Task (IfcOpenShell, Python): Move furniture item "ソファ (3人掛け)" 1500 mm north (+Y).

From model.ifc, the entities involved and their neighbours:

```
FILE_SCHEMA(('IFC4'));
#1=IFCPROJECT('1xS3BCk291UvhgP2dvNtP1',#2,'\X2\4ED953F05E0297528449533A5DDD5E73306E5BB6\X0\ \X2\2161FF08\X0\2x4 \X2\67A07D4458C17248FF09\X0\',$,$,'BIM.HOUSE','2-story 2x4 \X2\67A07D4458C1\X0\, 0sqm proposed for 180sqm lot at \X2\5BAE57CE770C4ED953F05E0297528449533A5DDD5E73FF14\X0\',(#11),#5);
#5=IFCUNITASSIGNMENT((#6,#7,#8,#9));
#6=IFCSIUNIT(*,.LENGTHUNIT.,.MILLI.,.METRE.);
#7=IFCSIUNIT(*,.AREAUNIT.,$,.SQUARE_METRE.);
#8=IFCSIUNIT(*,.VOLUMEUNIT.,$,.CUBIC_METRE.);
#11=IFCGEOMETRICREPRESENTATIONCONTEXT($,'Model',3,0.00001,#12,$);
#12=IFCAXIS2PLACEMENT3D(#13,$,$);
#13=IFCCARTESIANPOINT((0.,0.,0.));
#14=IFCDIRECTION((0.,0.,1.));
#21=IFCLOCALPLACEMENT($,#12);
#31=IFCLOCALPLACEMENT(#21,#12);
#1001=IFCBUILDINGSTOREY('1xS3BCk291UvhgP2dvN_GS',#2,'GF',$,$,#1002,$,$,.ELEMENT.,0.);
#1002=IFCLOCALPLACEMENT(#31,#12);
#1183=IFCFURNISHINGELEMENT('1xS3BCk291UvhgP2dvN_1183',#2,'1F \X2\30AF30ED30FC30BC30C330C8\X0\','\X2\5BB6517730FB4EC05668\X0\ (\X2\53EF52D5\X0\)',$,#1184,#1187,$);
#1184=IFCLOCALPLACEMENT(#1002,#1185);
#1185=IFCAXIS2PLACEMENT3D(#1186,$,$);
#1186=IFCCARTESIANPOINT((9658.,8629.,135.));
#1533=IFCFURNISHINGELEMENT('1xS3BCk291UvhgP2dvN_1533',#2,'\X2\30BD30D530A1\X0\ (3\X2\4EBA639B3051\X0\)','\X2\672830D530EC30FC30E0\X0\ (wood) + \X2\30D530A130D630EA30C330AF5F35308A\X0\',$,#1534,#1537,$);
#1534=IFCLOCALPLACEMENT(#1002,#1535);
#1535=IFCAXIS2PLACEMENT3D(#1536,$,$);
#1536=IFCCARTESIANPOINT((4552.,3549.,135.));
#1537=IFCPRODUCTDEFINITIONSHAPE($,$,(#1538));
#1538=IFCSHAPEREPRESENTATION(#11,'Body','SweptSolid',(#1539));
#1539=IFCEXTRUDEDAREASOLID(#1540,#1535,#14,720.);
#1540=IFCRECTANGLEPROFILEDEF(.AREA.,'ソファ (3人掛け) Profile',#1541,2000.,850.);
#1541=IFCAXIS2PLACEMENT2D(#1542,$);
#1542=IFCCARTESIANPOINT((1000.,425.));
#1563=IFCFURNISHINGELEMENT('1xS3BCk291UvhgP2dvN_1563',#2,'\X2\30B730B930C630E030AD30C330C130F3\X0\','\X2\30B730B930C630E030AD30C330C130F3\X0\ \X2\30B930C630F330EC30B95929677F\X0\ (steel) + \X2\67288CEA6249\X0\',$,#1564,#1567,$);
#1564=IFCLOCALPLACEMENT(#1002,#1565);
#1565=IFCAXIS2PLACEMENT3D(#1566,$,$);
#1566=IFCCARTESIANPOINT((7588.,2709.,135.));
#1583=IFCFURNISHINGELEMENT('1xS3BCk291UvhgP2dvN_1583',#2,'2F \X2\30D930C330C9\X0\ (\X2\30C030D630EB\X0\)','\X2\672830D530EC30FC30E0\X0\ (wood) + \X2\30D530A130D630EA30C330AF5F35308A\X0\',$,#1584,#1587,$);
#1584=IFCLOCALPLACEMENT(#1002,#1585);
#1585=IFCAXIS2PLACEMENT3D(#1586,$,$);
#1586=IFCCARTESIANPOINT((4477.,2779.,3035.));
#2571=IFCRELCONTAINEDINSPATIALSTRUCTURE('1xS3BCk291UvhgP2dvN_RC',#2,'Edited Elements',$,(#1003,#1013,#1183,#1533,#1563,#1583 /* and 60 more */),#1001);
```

```python
import ifcopenshell
import ifcopenshell.api.geometry
import ifcopenshell.util.placement

model = ifcopenshell.open("model.ifc")

item = model.by_guid("1xS3BCk291UvhgP2dvN_1533")
matrix = ifcopenshell.util.placement.get_local_placement(item.ObjectPlacement)
matrix[1, 3] += 1500.0
ifcopenshell.api.geometry.edit_object_placement(model, product=item, matrix=matrix, is_si=False)

print(ifcopenshell.util.placement.get_local_placement(item.ObjectPlacement).round(3) + 0.0)

model.write("model_edited.ifc")
```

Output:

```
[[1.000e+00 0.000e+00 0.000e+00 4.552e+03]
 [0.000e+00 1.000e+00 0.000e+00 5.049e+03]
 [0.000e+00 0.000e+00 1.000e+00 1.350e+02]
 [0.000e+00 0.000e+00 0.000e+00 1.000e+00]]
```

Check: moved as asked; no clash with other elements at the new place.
